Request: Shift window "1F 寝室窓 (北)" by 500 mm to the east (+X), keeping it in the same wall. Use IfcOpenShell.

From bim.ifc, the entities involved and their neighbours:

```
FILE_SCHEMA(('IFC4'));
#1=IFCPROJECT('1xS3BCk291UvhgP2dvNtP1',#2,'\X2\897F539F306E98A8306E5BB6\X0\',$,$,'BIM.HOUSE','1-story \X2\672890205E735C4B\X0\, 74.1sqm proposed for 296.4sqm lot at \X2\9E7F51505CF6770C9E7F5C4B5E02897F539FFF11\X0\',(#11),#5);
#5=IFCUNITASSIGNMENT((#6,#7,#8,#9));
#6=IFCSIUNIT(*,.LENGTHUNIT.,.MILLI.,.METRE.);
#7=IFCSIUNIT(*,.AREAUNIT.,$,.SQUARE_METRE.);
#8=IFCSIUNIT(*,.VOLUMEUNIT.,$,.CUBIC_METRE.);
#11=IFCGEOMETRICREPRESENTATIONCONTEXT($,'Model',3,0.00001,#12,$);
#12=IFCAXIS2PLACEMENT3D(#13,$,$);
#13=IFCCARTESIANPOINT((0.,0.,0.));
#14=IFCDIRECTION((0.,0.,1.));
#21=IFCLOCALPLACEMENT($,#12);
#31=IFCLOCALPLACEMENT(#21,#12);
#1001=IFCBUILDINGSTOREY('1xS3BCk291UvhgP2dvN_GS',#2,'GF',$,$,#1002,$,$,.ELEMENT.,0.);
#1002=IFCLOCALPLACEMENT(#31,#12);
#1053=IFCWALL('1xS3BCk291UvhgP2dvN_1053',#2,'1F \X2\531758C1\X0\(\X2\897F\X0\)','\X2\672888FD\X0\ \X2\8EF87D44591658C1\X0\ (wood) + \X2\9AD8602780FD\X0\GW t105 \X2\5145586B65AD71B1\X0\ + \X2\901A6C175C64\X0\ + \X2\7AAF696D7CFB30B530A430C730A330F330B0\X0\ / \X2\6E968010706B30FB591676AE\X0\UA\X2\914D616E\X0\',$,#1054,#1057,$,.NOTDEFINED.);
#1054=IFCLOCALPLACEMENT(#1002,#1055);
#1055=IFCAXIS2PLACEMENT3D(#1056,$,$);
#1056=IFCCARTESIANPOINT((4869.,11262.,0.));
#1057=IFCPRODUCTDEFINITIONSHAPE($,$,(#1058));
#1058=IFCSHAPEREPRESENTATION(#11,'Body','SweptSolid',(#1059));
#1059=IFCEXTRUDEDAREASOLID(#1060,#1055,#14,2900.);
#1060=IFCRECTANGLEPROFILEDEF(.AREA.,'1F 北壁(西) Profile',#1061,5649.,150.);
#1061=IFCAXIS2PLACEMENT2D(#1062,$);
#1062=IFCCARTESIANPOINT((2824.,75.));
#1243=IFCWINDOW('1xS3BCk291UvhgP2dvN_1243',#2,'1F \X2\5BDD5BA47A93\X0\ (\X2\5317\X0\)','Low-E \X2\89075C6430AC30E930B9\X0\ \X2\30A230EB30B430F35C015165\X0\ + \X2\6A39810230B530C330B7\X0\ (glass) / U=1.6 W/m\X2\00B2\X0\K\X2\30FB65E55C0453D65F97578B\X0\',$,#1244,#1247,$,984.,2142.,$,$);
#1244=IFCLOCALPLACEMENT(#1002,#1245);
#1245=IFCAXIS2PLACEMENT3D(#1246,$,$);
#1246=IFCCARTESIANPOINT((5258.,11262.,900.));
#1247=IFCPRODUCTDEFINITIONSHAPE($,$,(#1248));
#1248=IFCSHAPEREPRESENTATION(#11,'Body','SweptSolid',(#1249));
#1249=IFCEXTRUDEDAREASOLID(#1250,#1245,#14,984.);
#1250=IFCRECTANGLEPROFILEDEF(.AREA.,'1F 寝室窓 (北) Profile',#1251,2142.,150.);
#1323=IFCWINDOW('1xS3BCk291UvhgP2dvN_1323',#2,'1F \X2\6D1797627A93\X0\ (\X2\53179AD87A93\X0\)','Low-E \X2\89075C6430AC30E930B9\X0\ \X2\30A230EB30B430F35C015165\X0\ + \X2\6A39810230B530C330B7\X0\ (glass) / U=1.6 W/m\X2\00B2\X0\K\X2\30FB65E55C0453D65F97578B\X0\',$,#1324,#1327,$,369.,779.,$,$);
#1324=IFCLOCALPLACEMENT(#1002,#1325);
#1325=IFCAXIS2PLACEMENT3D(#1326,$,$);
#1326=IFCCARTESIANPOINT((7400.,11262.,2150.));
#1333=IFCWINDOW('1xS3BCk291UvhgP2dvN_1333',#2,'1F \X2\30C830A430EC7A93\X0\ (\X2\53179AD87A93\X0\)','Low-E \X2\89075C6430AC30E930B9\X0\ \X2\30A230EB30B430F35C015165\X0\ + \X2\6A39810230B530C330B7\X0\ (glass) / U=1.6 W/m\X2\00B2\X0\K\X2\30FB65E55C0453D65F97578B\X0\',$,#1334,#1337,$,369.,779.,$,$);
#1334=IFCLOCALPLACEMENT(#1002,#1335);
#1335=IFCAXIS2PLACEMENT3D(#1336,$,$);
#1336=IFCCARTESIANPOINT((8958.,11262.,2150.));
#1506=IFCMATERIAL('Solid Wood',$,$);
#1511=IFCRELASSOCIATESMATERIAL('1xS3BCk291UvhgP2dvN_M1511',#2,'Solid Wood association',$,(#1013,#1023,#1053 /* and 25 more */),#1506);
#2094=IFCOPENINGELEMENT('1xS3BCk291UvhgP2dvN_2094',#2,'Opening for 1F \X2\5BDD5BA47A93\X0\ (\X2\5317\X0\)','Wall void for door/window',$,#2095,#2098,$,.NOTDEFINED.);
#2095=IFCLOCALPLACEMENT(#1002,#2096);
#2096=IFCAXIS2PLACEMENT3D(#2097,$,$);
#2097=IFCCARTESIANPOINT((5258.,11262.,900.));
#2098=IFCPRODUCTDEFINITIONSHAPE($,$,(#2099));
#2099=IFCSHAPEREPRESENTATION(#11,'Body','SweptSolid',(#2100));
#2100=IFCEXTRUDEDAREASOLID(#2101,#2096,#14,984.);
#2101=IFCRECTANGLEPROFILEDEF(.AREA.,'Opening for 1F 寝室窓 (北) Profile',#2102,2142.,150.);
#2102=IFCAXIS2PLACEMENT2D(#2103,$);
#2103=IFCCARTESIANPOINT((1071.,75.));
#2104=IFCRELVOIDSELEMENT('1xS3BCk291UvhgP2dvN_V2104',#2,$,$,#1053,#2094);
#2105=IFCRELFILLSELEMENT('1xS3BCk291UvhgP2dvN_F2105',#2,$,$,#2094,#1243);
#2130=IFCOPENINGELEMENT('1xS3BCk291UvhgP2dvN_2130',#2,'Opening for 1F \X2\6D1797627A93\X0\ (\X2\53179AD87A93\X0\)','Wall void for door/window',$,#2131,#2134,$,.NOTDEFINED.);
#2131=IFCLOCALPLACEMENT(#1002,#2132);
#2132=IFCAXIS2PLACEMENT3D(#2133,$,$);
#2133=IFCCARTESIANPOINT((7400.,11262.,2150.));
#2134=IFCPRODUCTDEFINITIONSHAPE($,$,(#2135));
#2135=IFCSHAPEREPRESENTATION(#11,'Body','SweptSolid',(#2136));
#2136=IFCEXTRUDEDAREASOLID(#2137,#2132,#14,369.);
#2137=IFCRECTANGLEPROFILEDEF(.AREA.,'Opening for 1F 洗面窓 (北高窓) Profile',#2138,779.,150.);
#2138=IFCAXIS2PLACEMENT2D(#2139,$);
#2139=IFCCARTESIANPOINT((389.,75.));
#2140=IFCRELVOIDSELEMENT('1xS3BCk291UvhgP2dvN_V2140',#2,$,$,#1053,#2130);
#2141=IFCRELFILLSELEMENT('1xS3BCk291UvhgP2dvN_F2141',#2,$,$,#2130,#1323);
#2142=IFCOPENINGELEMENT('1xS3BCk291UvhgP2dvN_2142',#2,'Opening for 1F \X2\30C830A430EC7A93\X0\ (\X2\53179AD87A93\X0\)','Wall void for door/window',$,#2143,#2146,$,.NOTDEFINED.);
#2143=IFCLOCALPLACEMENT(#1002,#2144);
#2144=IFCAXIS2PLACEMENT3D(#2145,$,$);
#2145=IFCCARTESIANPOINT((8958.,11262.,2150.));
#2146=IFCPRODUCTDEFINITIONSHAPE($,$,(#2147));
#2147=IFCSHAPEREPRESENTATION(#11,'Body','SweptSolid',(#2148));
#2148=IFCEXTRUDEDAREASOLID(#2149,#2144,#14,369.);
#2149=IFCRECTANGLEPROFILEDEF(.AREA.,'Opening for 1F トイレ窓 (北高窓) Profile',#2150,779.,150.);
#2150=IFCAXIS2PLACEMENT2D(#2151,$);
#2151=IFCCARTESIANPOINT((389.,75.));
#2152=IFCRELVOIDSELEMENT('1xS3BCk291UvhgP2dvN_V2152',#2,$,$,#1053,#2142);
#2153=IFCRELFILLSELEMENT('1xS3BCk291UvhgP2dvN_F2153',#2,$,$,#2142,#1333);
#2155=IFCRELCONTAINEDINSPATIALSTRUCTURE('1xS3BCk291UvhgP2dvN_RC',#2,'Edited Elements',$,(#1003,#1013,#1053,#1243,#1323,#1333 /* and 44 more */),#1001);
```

```python
import ifcopenshell
import ifcopenshell.api.geometry
import ifcopenshell.util.placement
import ifcopenshell.util.unit

model = ifcopenshell.open("bim.ifc")
unit_scale = ifcopenshell.util.unit.calculate_unit_scale(model)

window = model.by_id(1243)
opening = window.FillsVoids[0].RelatingOpeningElement
wall = opening.VoidsElements[0].RelatingBuildingElement

wall_matrix = ifcopenshell.util.placement.get_local_placement(wall.ObjectPlacement)
shift = wall_matrix[:3, 0] * 0.5 / unit_scale
before = ifcopenshell.util.placement.get_local_placement(window.ObjectPlacement)[:3, 3].copy()

# The window is not placed relative to its opening, so move both.
for product in (opening, window):
    matrix = ifcopenshell.util.placement.get_local_placement(product.ObjectPlacement)
    matrix[:3, 3] += shift
    ifcopenshell.api.geometry.edit_object_placement(model, product=product, matrix=matrix, is_si=False)

after = ifcopenshell.util.placement.get_local_placement(window.ObjectPlacement)[:3, 3]
print("window moved by", (after - before).round(3) + 0.0)

model.write("bim_v2.ifc")
```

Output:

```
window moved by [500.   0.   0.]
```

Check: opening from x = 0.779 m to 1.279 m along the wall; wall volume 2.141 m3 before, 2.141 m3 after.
